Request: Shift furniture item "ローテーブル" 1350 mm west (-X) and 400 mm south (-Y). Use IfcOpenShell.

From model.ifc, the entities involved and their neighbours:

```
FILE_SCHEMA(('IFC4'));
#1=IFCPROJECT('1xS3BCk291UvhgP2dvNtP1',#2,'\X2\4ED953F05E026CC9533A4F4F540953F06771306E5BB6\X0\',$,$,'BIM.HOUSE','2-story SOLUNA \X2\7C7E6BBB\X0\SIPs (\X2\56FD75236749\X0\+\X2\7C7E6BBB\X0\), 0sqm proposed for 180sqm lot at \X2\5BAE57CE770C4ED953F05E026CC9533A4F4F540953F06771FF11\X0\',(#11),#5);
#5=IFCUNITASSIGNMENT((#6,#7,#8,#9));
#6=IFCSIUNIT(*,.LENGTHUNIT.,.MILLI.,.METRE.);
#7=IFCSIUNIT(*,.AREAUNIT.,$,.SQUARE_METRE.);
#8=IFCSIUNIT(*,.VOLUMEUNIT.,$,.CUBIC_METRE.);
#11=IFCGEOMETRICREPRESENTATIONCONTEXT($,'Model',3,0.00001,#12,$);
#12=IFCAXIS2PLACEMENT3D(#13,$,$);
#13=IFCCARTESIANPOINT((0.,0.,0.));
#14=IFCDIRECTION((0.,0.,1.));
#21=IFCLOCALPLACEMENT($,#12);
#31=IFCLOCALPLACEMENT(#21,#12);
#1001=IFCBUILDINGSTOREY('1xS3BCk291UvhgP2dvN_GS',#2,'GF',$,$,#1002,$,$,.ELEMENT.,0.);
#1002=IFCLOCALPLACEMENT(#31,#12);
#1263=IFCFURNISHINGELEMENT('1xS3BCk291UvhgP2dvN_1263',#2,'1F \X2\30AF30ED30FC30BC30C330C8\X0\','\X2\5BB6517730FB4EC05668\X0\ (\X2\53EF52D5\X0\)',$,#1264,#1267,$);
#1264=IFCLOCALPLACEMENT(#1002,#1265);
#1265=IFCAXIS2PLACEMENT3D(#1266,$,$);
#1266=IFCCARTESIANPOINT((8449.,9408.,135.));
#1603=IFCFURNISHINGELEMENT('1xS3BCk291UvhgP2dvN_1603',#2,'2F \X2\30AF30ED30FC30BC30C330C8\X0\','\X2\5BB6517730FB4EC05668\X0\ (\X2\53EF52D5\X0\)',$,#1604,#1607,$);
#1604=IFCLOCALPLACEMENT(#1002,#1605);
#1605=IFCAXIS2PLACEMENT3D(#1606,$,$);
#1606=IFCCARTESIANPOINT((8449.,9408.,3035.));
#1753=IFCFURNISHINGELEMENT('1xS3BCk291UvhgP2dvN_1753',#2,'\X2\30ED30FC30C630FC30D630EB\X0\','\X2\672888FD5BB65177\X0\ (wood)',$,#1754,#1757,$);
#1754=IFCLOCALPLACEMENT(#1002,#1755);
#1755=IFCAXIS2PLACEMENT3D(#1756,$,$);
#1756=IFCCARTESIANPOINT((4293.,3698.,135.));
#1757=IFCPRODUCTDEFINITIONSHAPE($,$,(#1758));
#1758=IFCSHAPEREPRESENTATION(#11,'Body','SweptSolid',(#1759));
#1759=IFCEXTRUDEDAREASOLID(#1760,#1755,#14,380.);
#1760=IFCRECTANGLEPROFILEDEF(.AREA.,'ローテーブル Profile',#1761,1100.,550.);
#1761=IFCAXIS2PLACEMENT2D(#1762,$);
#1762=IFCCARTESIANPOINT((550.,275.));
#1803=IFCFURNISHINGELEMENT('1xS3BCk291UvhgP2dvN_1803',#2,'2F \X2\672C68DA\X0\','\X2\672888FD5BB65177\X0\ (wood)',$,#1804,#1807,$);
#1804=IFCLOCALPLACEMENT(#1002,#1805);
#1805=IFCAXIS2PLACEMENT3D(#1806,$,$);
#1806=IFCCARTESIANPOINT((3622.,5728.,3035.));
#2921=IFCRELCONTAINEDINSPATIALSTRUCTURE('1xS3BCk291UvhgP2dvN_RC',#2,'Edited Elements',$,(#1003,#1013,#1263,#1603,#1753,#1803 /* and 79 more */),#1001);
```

```python
import ifcopenshell
import ifcopenshell.api.geometry
import ifcopenshell.util.placement
import ifcopenshell.util.unit

model = ifcopenshell.open("model.ifc")
unit_scale = ifcopenshell.util.unit.calculate_unit_scale(model)

item = model.by_guid("1xS3BCk291UvhgP2dvN_1753")
matrix = ifcopenshell.util.placement.get_local_placement(item.ObjectPlacement)
matrix[0, 3] -= 1.35 / unit_scale
matrix[1, 3] -= 0.4 / unit_scale
ifcopenshell.api.geometry.edit_object_placement(model, product=item, matrix=matrix, is_si=False)

print(ifcopenshell.util.placement.get_local_placement(item.ObjectPlacement).round(3) + 0.0)

model.write("model_rev.ifc")
```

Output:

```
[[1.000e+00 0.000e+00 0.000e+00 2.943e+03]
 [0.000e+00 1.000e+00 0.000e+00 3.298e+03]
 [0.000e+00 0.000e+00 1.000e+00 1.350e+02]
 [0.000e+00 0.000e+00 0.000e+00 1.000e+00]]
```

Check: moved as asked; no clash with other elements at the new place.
